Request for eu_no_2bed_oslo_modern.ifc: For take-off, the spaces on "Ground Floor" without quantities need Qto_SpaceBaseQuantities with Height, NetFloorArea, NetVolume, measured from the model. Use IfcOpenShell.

First a look at what the model holds.

```python
import ifcopenshell
import ifcopenshell.util.element
import ifcopenshell.util.unit

model = ifcopenshell.open("eu_no_2bed_oslo_modern.ifc")
print(model.schema)
for unit_type in ("LENGTHUNIT", "AREAUNIT", "VOLUMEUNIT"):
    print(unit_type, ifcopenshell.util.unit.calculate_unit_scale(model, unit_type))
storey = next(s for s in model.by_type("IfcBuildingStorey") if s.Name == "Ground Floor")
spaces = [e for e in ifcopenshell.util.element.get_decomposition(storey) if e.is_a("IfcSpace")]
for e in sorted(spaces, key=lambda e: e.id()):
    print(e.id(), e.is_a(), e.Name, list(ifcopenshell.util.element.get_psets(e, qtos_only=True)), sep=" | ")
```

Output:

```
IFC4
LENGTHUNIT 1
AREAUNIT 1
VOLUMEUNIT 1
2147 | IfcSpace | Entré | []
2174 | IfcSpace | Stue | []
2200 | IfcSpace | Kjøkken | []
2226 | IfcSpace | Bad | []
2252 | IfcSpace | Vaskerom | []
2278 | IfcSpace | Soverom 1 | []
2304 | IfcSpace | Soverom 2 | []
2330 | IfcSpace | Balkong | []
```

```python
import ifcopenshell
import ifcopenshell.api.pset
import ifcopenshell.geom
import ifcopenshell.util.element
import ifcopenshell.util.shape
import ifcopenshell.util.unit

model = ifcopenshell.open("eu_no_2bed_oslo_modern.ifc")
unit_scale = ifcopenshell.util.unit.calculate_unit_scale(model)
area_scale = ifcopenshell.util.unit.calculate_unit_scale(model, "AREAUNIT")
volume_scale = ifcopenshell.util.unit.calculate_unit_scale(model, "VOLUMEUNIT")
settings = ifcopenshell.geom.settings()

storey = next(s for s in model.by_type("IfcBuildingStorey") if s.Name == "Ground Floor")
spaces = [e for e in ifcopenshell.util.element.get_decomposition(storey) if e.is_a("IfcSpace")]

for e in sorted(spaces, key=lambda e: e.id()):
    if ifcopenshell.util.element.get_psets(e, qtos_only=True, should_inherit=False):
        continue
    # Geometry comes back in metres, in the element's own axes.
    shape = ifcopenshell.geom.create_shape(settings, e)
    values = {
        "Height": ifcopenshell.util.shape.get_z(shape.geometry) / unit_scale,
        "NetFloorArea": ifcopenshell.util.shape.get_footprint_area(shape.geometry) / area_scale,
        "NetVolume": ifcopenshell.util.shape.get_volume(shape.geometry) / volume_scale,
    }
    qto = ifcopenshell.api.pset.add_qto(model, product=e, name="Qto_SpaceBaseQuantities")
    ifcopenshell.api.pset.edit_qto(model, qto=qto, properties=values)
    print(e.id(), {k: round(v, 3) for k, v in values.items()})

model.write("eu_no_2bed_oslo_modern_rev.ifc")
```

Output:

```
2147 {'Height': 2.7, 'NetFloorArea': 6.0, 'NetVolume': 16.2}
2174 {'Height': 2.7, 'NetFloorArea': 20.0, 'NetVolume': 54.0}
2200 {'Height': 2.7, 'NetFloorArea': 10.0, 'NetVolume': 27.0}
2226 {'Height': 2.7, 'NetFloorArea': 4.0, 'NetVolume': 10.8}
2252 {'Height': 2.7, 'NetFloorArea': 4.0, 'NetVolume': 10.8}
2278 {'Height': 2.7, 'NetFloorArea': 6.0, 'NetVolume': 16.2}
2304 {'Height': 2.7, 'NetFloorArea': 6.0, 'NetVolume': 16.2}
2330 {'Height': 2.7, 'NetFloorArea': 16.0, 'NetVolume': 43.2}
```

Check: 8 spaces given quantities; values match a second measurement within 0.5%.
